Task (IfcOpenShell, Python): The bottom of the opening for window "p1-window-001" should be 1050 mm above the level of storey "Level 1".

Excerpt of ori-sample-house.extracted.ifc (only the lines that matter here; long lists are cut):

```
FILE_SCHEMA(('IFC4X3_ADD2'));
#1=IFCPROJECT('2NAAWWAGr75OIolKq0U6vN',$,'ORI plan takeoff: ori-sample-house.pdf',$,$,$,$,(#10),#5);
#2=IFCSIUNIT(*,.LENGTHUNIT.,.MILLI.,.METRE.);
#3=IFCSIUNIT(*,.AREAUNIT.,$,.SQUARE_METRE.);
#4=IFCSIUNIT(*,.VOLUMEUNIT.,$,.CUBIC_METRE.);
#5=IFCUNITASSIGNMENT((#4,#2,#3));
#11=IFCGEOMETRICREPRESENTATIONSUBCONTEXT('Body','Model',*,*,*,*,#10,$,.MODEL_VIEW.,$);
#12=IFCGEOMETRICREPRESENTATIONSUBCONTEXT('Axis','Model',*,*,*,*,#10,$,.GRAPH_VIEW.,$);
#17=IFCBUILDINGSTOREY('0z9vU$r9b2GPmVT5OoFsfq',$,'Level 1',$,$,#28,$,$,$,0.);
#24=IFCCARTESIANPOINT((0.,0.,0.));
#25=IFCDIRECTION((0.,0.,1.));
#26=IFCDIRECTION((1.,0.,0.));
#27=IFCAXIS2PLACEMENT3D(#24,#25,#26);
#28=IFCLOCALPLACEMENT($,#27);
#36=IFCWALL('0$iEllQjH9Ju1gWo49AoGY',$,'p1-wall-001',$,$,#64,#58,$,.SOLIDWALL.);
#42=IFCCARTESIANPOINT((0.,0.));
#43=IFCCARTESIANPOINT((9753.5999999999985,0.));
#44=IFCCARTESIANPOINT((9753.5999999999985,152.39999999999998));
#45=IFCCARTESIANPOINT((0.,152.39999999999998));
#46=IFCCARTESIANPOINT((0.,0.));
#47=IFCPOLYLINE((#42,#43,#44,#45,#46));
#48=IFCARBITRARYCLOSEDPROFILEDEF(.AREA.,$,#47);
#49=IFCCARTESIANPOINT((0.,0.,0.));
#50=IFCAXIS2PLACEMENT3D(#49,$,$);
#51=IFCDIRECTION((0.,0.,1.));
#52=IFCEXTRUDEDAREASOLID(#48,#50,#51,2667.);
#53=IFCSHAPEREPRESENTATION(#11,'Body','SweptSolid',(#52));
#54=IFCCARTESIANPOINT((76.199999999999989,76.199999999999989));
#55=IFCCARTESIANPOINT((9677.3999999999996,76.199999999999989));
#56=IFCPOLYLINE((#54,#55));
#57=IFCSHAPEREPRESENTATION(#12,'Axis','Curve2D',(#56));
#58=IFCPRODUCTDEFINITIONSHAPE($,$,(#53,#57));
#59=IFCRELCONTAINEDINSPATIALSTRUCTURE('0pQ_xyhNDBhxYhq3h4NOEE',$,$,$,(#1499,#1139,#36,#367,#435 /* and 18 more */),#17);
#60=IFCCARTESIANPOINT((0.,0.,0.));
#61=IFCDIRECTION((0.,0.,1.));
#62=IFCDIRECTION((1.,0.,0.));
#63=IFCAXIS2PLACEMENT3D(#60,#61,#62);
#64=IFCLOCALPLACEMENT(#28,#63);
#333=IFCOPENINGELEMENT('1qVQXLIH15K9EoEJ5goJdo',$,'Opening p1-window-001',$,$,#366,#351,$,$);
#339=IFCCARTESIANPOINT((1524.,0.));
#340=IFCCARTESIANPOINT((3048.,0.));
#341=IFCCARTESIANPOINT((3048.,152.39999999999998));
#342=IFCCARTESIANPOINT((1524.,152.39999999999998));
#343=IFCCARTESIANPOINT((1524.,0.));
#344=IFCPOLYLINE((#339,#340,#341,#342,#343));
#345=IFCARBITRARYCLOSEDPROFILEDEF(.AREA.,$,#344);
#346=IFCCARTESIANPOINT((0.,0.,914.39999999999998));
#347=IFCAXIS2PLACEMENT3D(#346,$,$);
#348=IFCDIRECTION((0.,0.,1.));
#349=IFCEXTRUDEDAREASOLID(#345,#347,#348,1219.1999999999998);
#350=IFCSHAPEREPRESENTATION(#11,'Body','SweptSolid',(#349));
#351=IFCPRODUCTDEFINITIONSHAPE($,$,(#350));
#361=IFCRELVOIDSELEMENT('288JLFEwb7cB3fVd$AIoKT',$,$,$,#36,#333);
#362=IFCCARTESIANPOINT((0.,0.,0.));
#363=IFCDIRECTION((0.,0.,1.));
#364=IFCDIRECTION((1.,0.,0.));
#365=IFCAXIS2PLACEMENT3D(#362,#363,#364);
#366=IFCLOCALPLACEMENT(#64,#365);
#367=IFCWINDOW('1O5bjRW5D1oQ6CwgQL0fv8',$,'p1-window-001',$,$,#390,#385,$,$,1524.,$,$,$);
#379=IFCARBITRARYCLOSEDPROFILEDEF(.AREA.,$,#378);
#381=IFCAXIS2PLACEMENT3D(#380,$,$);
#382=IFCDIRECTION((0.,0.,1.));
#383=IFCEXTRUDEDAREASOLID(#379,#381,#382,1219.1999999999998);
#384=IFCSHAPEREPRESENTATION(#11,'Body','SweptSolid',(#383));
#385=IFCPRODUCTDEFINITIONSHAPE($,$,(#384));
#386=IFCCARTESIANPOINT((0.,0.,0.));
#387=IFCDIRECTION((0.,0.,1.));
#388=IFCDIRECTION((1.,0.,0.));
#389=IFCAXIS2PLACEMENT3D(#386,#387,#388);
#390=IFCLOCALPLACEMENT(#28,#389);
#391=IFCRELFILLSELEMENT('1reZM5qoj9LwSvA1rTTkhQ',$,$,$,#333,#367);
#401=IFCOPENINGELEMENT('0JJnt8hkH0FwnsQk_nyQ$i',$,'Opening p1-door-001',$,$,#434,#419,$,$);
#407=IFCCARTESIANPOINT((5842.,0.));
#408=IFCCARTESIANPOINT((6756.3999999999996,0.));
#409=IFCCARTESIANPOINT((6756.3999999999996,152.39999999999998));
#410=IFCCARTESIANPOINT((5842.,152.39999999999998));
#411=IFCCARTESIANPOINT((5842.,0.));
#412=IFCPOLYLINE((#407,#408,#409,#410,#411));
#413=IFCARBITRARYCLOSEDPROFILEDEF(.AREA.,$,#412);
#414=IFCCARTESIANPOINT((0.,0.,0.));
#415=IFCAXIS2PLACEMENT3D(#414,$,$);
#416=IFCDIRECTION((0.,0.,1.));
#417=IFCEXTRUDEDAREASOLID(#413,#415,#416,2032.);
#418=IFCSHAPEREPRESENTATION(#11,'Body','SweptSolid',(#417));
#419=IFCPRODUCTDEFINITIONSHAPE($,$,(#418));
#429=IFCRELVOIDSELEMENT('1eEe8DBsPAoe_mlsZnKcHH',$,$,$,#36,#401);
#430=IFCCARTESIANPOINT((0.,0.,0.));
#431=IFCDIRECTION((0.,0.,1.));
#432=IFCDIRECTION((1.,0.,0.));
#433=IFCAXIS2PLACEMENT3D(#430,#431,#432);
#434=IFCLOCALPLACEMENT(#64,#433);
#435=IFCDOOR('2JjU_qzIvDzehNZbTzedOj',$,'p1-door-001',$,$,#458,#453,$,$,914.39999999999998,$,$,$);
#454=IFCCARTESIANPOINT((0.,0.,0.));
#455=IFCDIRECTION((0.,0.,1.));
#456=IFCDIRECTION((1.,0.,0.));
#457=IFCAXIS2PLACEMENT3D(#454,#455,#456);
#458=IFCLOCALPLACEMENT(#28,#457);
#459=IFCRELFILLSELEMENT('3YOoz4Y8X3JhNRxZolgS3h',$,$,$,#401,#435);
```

```python
import numpy as np
import ifcopenshell
import ifcopenshell.api.geometry
import ifcopenshell.geom
import ifcopenshell.util.element
import ifcopenshell.util.placement
import ifcopenshell.util.shape
import ifcopenshell.util.unit

model = ifcopenshell.open("ori-sample-house.extracted.ifc")
unit_scale = ifcopenshell.util.unit.calculate_unit_scale(model)

window = model.by_guid("1O5bjRW5D1oQ6CwgQL0fv8")
opening = window.FillsVoids[0].RelatingOpeningElement
storey = ifcopenshell.util.element.get_container(window, ifc_class="IfcBuildingStorey")
level = ifcopenshell.util.placement.get_local_placement(storey.ObjectPlacement)[2, 3]

# The opening's origin need not be at the sill, so measure its lowest point.
shape = ifcopenshell.geom.create_shape(ifcopenshell.geom.settings(), opening)
bottom = ifcopenshell.util.shape.get_shape_bottom_elevation(shape, shape.geometry) / unit_scale
dz = level + 1.05 / unit_scale - bottom

shift = np.array([0.0, 0.0, dz])
# The window is not placed relative to its opening, so move both.
for product in (opening, window):
    matrix = ifcopenshell.util.placement.get_local_placement(product.ObjectPlacement)
    matrix[:3, 3] += shift
    ifcopenshell.api.geometry.edit_object_placement(model, product=product, matrix=matrix, is_si=False)

print(f"moved by {dz * unit_scale:+.3f} m")

model.write("ori-sample-house.extracted_updated.ifc")
```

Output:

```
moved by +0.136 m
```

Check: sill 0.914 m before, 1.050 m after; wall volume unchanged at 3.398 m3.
